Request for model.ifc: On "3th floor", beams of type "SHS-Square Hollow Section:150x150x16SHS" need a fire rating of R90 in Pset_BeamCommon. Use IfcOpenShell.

First a look at what the model holds.

```python
import ifcopenshell
import ifcopenshell.util.element

model = ifcopenshell.open("model.ifc")
print(model.schema)
storey = next(s for s in model.by_type("IfcBuildingStorey") if s.Name == "3th floor")
beams = [e for e in ifcopenshell.util.element.get_decomposition(storey) if e.is_a("IfcBeam")]
seen = {}
for e in beams:
    element_type = ifcopenshell.util.element.get_type(e)
    key = (element_type.Name if element_type != e and element_type else None, ifcopenshell.util.element.get_pset(e, "Pset_BeamCommon", "FireRating"))
    seen[key] = seen.get(key, 0) + 1
for (name, value), count in sorted(seen.items(), key=str):
    print(count, "x", name, "|", value)
```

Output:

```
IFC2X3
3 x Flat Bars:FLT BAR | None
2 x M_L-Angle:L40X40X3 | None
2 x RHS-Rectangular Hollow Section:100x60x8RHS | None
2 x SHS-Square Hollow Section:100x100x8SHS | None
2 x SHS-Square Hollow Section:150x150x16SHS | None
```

```python
import ifcopenshell
import ifcopenshell.api.pset
import ifcopenshell.util.element

model = ifcopenshell.open("model.ifc")

storey = next(s for s in model.by_type("IfcBuildingStorey") if s.Name == "3th floor")
beams = [e for e in ifcopenshell.util.element.get_decomposition(storey) if e.is_a("IfcBeam")]

count = 0
for e in beams:
    element_type = ifcopenshell.util.element.get_type(e)
    if element_type in (None, e) or element_type.Name != "SHS-Square Hollow Section:150x150x16SHS":
        continue
    # add_pset returns the element's existing set when there is one.
    pset = ifcopenshell.api.pset.add_pset(model, product=e, name="Pset_BeamCommon")
    ifcopenshell.api.pset.edit_pset(model, pset=pset, properties={"FireRating": "R90"})
    count += 1

print(count, "beams updated")

model.write("model_edited.ifc")
```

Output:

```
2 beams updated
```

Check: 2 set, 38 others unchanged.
